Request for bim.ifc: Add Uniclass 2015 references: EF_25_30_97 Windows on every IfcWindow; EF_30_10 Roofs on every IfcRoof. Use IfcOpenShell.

First a look at what the model holds.

```python
import ifcopenshell

model = ifcopenshell.open("bim.ifc")
print(model.schema)
print("classifications:", [c.Name for c in model.by_type("IfcClassification")])
for ifc_class in ("IfcDoor", "IfcRoof", "IfcStair", "IfcWall", "IfcWindow"):
    print(ifc_class, len(model.by_type(ifc_class)))
```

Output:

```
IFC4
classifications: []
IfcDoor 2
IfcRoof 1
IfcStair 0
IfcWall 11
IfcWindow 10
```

```python
import ifcopenshell
import ifcopenshell.api.classification

model = ifcopenshell.open("bim.ifc")

system = ifcopenshell.api.classification.add_classification(model, classification="Uniclass 2015")

codes = {
    "IfcWindow": ("EF_25_30_97", "Windows"),
    "IfcRoof": ("EF_30_10", "Roofs"),
}
for ifc_class, (code, name) in codes.items():
    products = model.by_type(ifc_class)
    ifcopenshell.api.classification.add_reference(
        model, products=products, classification=system, identification=code, name=name
    )
    print(code, len(products))

model.write("bim-out.ifc")
```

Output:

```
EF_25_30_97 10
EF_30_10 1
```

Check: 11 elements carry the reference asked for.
